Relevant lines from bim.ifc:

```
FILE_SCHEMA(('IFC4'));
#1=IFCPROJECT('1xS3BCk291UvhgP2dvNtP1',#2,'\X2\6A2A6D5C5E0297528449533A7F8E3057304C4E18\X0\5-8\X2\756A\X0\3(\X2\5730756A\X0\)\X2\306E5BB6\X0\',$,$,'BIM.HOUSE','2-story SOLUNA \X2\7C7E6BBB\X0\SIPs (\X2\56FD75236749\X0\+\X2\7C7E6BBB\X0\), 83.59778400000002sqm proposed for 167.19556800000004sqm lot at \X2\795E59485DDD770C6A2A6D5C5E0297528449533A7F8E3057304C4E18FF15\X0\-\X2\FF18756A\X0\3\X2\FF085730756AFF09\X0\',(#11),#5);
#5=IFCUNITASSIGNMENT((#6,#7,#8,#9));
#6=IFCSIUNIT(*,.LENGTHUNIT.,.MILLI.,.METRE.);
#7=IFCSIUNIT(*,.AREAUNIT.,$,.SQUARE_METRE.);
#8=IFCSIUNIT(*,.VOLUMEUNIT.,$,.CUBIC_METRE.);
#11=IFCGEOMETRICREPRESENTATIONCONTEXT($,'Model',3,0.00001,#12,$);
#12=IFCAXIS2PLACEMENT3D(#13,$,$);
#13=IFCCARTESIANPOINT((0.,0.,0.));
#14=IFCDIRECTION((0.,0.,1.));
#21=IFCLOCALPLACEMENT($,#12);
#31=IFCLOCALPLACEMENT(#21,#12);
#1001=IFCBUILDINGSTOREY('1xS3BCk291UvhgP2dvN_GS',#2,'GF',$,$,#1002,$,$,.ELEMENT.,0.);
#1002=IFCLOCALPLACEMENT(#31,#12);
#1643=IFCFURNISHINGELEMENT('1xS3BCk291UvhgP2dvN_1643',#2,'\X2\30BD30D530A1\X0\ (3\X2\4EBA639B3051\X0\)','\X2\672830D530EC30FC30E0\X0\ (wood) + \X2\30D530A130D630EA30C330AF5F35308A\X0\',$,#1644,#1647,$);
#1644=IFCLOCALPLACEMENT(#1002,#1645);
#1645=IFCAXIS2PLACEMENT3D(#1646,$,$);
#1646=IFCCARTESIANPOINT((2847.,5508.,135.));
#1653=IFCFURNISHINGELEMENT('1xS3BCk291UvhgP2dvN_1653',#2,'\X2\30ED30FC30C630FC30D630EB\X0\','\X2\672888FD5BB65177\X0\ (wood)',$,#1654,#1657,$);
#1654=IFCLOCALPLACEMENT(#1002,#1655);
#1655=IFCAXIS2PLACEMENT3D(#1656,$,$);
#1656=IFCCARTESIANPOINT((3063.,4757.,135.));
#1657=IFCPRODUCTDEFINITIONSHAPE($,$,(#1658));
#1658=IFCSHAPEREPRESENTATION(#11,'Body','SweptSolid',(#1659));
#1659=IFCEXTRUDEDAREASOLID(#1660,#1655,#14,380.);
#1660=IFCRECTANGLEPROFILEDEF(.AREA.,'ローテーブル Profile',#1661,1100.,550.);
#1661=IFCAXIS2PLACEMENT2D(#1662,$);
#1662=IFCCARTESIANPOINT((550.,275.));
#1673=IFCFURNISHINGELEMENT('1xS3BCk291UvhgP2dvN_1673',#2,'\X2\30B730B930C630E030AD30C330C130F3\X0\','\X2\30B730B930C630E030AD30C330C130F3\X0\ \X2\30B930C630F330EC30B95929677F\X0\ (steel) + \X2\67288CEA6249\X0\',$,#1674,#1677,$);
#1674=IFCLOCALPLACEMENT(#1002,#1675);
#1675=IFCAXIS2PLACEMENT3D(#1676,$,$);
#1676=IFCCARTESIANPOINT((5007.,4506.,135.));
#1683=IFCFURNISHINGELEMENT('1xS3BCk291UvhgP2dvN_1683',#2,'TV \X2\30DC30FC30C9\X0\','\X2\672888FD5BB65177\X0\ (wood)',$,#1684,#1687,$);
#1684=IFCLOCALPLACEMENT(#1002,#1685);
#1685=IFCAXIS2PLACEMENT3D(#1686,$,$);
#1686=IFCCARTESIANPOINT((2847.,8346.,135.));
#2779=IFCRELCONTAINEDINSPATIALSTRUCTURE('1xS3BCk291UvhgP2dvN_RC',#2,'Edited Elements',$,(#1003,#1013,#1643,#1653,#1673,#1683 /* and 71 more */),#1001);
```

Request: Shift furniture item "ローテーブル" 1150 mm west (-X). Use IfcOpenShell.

```python
import ifcopenshell
import ifcopenshell.api.geometry
import ifcopenshell.util.placement
import ifcopenshell.util.unit

model = ifcopenshell.open("bim.ifc")
unit_scale = ifcopenshell.util.unit.calculate_unit_scale(model)

item = model.by_guid("1xS3BCk291UvhgP2dvN_1653")
matrix = ifcopenshell.util.placement.get_local_placement(item.ObjectPlacement)
matrix[0, 3] -= 1.15 / unit_scale
ifcopenshell.api.geometry.edit_object_placement(model, product=item, matrix=matrix, is_si=False)

print(ifcopenshell.util.placement.get_local_placement(item.ObjectPlacement).round(3) + 0.0)

model.write("bim_updated.ifc")
```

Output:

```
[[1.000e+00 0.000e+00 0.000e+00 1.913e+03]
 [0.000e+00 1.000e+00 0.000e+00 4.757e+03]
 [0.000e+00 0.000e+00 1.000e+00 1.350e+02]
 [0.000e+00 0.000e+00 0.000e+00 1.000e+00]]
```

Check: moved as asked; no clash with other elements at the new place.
